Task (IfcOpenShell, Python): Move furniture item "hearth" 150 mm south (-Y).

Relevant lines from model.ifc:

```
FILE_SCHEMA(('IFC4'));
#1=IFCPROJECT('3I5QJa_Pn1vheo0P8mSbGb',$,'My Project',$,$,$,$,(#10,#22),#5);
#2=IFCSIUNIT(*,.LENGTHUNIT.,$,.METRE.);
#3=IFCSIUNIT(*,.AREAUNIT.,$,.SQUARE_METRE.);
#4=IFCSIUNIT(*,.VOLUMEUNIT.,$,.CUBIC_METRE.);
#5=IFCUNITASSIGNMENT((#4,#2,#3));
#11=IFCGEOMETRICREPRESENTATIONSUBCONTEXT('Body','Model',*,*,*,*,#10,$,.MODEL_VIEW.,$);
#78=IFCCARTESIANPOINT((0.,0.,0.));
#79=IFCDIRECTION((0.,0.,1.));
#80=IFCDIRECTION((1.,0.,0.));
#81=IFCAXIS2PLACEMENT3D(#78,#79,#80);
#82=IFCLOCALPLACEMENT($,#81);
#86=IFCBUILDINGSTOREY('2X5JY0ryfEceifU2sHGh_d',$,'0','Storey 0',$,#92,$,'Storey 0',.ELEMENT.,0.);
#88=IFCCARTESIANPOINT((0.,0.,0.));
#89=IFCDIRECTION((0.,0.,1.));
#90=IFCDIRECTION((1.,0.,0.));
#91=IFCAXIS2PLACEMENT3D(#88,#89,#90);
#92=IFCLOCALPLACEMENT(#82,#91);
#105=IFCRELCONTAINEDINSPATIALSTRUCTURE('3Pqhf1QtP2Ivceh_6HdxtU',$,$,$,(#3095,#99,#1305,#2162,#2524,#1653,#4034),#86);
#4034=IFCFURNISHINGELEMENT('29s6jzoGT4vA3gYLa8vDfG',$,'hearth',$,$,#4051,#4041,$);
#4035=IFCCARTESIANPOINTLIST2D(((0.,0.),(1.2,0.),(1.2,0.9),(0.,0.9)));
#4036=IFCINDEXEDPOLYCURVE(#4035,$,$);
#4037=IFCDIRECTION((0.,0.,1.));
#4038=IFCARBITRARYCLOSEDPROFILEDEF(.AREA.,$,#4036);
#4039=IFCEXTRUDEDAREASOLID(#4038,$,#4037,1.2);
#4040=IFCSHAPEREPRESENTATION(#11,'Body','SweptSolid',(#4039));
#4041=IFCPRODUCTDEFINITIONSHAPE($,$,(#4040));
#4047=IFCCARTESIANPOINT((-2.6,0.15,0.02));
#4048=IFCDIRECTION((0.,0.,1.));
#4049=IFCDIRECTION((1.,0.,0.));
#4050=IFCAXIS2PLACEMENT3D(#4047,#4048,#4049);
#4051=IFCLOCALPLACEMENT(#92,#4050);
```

```python
import ifcopenshell
import ifcopenshell.api.geometry
import ifcopenshell.util.placement

model = ifcopenshell.open("model.ifc")

item = model.by_guid("29s6jzoGT4vA3gYLa8vDfG")
matrix = ifcopenshell.util.placement.get_local_placement(item.ObjectPlacement)
matrix[1, 3] -= 0.15
ifcopenshell.api.geometry.edit_object_placement(model, product=item, matrix=matrix, is_si=False)

print(ifcopenshell.util.placement.get_local_placement(item.ObjectPlacement).round(3) + 0.0)

model.write("model_v2.ifc")
```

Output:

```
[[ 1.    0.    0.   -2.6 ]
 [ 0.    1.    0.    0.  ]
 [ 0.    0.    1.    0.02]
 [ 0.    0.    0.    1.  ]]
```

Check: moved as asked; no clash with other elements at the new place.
